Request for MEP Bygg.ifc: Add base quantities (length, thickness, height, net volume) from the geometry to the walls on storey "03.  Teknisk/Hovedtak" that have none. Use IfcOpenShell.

First a look at what the model holds.

```python
import ifcopenshell
import ifcopenshell.util.element
import ifcopenshell.util.unit

model = ifcopenshell.open("MEP Bygg.ifc")
print(model.schema)
for unit_type in ("LENGTHUNIT", "AREAUNIT", "VOLUMEUNIT"):
    print(unit_type, ifcopenshell.util.unit.calculate_unit_scale(model, unit_type))
storey = next(s for s in model.by_type("IfcBuildingStorey") if s.Name == "03.  Teknisk/Hovedtak")
walls = [e for e in ifcopenshell.util.element.get_decomposition(storey) if e.is_a("IfcWall")]
for e in sorted(walls, key=lambda e: e.id()):
    print(e.id(), e.is_a(), e.Name, list(ifcopenshell.util.element.get_psets(e, qtos_only=True)), sep=" | ")
```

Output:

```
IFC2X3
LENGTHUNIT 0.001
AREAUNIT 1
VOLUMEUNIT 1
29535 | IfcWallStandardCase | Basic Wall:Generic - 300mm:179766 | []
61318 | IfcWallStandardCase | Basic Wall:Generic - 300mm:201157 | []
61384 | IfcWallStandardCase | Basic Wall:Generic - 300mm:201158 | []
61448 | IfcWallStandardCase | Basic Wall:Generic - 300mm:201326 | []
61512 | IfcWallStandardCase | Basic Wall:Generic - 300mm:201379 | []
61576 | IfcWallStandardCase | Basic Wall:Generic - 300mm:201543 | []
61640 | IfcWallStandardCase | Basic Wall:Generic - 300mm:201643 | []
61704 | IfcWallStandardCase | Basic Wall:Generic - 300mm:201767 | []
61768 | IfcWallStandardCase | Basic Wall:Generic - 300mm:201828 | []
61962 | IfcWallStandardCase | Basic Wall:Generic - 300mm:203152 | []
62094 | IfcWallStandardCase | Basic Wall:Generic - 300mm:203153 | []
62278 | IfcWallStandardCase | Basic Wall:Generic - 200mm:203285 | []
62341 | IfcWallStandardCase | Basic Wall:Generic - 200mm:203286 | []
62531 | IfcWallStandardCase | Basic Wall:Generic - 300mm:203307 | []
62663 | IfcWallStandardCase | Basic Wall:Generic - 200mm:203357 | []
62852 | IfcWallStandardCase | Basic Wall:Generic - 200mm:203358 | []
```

```python
import ifcopenshell
import ifcopenshell.api.pset
import ifcopenshell.geom
import ifcopenshell.util.element
import ifcopenshell.util.shape
import ifcopenshell.util.unit

model = ifcopenshell.open("MEP Bygg.ifc")
unit_scale = ifcopenshell.util.unit.calculate_unit_scale(model)
volume_scale = ifcopenshell.util.unit.calculate_unit_scale(model, "VOLUMEUNIT")
settings = ifcopenshell.geom.settings()

storey = next(s for s in model.by_type("IfcBuildingStorey") if s.Name == "03.  Teknisk/Hovedtak")
walls = [e for e in ifcopenshell.util.element.get_decomposition(storey) if e.is_a("IfcWall")]

for e in sorted(walls, key=lambda e: e.id()):
    if ifcopenshell.util.element.get_psets(e, qtos_only=True, should_inherit=False):
        continue
    # Geometry comes back in metres, in the element's own axes.
    shape = ifcopenshell.geom.create_shape(settings, e)
    values = {
        "Length": ifcopenshell.util.shape.get_x(shape.geometry) / unit_scale,
        "Width": ifcopenshell.util.shape.get_y(shape.geometry) / unit_scale,
        "Height": ifcopenshell.util.shape.get_z(shape.geometry) / unit_scale,
        "NetVolume": ifcopenshell.util.shape.get_volume(shape.geometry) / volume_scale,
    }
    qto = ifcopenshell.api.pset.add_qto(model, product=e, name="BaseQuantities")
    ifcopenshell.api.pset.edit_qto(model, qto=qto, properties=values)
    print(e.id(), {k: round(v, 3) for k, v in values.items()})

model.write("MEP Bygg_updated.ifc")
```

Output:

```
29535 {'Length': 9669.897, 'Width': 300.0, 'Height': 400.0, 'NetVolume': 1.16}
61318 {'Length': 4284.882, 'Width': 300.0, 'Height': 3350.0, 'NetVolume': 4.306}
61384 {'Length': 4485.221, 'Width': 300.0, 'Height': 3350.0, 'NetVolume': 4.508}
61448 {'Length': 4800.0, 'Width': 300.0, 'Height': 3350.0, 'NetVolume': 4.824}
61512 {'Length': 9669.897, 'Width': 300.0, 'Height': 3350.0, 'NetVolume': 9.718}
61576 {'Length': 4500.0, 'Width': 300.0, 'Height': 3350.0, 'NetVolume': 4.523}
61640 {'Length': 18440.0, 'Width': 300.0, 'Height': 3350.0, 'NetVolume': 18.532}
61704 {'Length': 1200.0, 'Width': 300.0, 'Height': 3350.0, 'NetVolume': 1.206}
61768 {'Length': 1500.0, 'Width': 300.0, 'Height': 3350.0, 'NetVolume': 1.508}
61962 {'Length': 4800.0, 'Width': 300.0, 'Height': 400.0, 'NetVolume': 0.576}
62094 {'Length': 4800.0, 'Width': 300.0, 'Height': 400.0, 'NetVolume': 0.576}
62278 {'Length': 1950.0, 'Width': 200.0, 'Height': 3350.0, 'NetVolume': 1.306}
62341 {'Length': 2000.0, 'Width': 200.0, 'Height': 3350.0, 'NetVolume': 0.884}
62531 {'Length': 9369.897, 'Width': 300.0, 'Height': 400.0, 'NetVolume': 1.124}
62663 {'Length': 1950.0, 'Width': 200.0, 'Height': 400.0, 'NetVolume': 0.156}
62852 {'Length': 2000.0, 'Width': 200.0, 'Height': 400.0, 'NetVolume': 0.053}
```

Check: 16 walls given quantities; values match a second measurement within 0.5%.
